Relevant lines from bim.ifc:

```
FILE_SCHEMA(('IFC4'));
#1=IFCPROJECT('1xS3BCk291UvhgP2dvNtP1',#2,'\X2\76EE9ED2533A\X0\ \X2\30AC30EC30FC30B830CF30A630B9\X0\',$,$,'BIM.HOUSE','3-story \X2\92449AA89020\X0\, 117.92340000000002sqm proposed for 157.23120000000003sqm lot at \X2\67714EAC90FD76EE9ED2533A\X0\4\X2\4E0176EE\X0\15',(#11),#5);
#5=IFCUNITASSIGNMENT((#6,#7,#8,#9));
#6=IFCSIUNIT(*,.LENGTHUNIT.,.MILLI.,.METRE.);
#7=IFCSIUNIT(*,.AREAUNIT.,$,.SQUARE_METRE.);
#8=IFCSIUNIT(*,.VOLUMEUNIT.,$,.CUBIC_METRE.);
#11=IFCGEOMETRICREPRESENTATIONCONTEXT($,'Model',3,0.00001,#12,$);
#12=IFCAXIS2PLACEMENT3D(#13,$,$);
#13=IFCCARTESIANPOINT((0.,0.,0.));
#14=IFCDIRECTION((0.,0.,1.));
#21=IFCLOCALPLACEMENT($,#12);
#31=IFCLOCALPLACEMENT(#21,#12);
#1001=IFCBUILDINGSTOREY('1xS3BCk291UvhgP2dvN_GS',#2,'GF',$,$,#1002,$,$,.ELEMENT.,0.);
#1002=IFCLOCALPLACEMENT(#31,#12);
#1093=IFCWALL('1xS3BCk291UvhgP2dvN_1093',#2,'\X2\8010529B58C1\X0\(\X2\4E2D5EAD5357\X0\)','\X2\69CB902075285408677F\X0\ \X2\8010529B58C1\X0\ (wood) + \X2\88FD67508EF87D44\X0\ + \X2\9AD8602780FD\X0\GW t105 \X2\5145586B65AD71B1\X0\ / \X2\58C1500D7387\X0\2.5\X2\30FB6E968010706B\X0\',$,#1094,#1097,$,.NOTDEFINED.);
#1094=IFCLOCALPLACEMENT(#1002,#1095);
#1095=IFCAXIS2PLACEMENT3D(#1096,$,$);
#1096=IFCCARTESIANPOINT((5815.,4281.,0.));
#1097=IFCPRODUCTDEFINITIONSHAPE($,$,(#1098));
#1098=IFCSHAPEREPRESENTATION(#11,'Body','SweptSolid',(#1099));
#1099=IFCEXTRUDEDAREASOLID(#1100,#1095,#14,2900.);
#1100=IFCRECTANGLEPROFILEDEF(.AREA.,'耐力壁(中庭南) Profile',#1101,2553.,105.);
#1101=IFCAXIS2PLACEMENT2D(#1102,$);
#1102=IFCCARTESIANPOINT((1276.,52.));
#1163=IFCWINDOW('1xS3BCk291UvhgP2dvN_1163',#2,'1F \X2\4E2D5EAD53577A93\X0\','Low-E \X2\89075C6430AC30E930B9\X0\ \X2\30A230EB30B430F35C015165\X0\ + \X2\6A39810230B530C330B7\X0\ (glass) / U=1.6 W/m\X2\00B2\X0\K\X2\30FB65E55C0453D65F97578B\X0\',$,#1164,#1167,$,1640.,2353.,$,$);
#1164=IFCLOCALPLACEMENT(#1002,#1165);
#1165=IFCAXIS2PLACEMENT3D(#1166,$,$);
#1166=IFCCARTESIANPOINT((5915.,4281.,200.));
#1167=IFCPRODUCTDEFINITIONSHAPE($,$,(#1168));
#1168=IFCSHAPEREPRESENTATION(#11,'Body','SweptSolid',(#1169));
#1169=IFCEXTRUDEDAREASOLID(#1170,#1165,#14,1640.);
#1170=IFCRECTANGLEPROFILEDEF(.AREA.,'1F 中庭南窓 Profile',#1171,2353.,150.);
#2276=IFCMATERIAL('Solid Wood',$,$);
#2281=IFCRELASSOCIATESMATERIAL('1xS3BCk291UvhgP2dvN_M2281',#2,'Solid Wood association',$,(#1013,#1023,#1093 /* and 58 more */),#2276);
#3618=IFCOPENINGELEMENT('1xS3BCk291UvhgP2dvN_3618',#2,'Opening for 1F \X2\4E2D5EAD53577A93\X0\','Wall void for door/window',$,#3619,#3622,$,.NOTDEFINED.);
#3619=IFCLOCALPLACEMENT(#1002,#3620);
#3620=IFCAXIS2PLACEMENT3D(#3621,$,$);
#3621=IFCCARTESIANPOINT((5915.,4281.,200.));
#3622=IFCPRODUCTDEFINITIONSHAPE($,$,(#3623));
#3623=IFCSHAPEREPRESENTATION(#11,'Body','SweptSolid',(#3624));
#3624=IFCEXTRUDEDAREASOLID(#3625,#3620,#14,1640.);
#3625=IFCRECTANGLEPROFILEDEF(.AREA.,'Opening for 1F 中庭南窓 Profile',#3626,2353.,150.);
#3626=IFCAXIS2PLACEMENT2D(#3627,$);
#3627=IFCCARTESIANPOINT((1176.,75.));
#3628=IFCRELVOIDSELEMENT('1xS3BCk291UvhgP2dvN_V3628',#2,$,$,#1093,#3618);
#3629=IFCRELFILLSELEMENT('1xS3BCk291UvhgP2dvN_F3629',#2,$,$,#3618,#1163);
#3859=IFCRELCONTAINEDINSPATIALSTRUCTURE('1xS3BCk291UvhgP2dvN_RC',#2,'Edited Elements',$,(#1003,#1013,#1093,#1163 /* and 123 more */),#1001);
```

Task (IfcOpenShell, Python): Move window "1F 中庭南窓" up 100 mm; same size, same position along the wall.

```python
import numpy as np
import ifcopenshell
import ifcopenshell.api.geometry
import ifcopenshell.util.placement
import ifcopenshell.util.unit

model = ifcopenshell.open("bim.ifc")
unit_scale = ifcopenshell.util.unit.calculate_unit_scale(model)

window = model.by_guid("1xS3BCk291UvhgP2dvN_1163")
opening = window.FillsVoids[0].RelatingOpeningElement
dz = 0.1 / unit_scale

shift = np.array([0.0, 0.0, dz])
# The window is not placed relative to its opening, so move both.
for product in (opening, window):
    matrix = ifcopenshell.util.placement.get_local_placement(product.ObjectPlacement)
    matrix[:3, 3] += shift
    ifcopenshell.api.geometry.edit_object_placement(model, product=product, matrix=matrix, is_si=False)

print(f"moved by {dz * unit_scale:+.3f} m")

model.write("bim_edited.ifc")
```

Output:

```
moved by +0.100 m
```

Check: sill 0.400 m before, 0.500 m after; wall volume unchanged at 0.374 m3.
